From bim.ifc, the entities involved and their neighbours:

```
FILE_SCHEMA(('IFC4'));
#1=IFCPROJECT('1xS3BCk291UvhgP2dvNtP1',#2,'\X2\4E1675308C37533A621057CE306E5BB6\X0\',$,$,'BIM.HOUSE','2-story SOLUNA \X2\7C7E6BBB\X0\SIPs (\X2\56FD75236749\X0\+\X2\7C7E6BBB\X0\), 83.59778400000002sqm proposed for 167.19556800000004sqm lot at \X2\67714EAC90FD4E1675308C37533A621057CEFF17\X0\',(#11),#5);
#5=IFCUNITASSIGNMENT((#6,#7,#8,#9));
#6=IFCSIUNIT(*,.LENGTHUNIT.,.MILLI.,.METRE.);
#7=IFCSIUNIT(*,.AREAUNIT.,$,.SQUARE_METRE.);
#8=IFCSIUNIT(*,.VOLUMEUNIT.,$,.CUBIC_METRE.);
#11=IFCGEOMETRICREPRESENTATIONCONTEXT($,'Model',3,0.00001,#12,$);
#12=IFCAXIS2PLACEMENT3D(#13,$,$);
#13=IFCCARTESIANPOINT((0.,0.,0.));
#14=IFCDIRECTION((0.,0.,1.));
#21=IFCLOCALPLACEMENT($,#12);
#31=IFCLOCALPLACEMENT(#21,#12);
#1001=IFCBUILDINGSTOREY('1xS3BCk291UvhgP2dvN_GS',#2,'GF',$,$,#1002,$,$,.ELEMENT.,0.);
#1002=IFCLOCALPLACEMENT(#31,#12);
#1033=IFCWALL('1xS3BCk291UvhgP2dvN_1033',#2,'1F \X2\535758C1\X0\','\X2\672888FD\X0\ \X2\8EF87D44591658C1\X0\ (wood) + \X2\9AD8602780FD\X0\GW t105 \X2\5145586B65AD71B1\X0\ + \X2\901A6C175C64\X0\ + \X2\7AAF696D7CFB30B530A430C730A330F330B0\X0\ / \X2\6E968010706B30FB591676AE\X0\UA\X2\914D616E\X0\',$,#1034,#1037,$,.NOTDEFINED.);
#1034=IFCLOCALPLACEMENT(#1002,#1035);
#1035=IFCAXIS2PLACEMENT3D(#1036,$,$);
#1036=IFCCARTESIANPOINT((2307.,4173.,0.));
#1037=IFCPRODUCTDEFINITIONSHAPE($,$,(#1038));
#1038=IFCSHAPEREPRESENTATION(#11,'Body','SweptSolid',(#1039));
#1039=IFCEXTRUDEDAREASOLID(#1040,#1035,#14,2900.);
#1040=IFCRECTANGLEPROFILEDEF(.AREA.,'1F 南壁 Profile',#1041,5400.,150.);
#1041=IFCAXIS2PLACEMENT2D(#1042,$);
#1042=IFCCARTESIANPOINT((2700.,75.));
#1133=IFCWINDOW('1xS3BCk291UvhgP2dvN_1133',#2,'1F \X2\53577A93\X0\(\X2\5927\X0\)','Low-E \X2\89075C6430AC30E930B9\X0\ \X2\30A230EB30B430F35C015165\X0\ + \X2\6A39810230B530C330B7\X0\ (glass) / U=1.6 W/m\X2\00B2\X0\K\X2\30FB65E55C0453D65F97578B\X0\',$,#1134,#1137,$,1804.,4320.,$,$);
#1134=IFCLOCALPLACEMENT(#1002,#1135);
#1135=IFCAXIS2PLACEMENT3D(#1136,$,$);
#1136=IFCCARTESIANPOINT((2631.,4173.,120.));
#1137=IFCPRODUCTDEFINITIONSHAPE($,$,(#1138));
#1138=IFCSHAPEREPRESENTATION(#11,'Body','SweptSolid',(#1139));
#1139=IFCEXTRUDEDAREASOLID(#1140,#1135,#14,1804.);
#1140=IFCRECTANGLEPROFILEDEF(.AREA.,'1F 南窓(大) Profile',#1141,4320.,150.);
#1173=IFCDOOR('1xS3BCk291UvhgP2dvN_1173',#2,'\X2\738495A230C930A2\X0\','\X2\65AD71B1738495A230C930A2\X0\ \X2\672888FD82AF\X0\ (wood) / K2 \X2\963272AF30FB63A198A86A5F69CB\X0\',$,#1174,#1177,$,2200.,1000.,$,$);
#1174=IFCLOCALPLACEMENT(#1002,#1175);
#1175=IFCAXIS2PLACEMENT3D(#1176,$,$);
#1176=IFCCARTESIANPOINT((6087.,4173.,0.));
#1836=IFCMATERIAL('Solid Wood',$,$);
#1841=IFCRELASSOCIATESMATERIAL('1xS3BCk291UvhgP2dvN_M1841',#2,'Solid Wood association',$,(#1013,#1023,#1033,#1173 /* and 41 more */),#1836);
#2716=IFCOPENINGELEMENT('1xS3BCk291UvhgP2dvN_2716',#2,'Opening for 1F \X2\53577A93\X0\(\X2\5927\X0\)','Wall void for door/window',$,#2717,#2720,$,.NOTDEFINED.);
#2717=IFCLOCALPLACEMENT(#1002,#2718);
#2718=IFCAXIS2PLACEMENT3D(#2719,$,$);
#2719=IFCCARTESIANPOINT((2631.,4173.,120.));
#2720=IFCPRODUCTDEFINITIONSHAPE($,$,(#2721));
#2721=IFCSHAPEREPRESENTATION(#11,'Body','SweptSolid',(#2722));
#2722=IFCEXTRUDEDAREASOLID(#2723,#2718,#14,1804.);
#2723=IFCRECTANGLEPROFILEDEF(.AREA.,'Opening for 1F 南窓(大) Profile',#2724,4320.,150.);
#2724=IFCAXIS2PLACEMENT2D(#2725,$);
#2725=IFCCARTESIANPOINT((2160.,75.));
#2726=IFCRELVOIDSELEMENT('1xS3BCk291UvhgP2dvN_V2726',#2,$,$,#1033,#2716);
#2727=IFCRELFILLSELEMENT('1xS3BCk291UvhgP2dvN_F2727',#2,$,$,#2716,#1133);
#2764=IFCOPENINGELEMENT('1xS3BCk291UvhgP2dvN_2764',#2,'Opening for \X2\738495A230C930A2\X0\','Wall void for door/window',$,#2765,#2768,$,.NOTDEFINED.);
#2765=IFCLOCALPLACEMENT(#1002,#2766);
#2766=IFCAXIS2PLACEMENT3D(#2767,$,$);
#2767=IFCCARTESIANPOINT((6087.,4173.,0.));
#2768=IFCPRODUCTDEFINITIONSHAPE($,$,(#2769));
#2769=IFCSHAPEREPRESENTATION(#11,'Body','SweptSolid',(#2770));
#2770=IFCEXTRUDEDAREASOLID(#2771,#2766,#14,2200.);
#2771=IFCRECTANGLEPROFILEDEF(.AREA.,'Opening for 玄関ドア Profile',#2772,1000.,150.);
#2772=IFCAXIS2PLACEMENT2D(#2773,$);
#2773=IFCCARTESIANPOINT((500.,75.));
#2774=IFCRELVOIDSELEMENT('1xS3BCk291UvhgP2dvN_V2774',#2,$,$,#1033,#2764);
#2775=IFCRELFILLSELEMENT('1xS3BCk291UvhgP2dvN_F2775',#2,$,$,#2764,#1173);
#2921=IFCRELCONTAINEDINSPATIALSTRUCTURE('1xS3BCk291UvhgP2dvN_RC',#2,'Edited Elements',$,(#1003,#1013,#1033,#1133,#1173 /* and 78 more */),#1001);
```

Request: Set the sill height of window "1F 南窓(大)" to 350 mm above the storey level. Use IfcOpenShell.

```python
import numpy as np
import ifcopenshell
import ifcopenshell.api.geometry
import ifcopenshell.geom
import ifcopenshell.util.element
import ifcopenshell.util.placement
import ifcopenshell.util.shape
import ifcopenshell.util.unit

model = ifcopenshell.open("bim.ifc")
unit_scale = ifcopenshell.util.unit.calculate_unit_scale(model)

window = model.by_guid("1xS3BCk291UvhgP2dvN_1133")
opening = window.FillsVoids[0].RelatingOpeningElement
storey = ifcopenshell.util.element.get_container(window, ifc_class="IfcBuildingStorey")
level = ifcopenshell.util.placement.get_local_placement(storey.ObjectPlacement)[2, 3]

# The opening's origin need not be at the sill, so measure its lowest point.
shape = ifcopenshell.geom.create_shape(ifcopenshell.geom.settings(), opening)
bottom = ifcopenshell.util.shape.get_shape_bottom_elevation(shape, shape.geometry) / unit_scale
dz = level + 350.0 - bottom

shift = np.array([0.0, 0.0, dz])
# The window is not placed relative to its opening, so move both.
for product in (opening, window):
    matrix = ifcopenshell.util.placement.get_local_placement(product.ObjectPlacement)
    matrix[:3, 3] += shift
    ifcopenshell.api.geometry.edit_object_placement(model, product=product, matrix=matrix, is_si=False)

print(f"moved by {dz * unit_scale:+.3f} m")

model.write("bim_edited.ifc")
```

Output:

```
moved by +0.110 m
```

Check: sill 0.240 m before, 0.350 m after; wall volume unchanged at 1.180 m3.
